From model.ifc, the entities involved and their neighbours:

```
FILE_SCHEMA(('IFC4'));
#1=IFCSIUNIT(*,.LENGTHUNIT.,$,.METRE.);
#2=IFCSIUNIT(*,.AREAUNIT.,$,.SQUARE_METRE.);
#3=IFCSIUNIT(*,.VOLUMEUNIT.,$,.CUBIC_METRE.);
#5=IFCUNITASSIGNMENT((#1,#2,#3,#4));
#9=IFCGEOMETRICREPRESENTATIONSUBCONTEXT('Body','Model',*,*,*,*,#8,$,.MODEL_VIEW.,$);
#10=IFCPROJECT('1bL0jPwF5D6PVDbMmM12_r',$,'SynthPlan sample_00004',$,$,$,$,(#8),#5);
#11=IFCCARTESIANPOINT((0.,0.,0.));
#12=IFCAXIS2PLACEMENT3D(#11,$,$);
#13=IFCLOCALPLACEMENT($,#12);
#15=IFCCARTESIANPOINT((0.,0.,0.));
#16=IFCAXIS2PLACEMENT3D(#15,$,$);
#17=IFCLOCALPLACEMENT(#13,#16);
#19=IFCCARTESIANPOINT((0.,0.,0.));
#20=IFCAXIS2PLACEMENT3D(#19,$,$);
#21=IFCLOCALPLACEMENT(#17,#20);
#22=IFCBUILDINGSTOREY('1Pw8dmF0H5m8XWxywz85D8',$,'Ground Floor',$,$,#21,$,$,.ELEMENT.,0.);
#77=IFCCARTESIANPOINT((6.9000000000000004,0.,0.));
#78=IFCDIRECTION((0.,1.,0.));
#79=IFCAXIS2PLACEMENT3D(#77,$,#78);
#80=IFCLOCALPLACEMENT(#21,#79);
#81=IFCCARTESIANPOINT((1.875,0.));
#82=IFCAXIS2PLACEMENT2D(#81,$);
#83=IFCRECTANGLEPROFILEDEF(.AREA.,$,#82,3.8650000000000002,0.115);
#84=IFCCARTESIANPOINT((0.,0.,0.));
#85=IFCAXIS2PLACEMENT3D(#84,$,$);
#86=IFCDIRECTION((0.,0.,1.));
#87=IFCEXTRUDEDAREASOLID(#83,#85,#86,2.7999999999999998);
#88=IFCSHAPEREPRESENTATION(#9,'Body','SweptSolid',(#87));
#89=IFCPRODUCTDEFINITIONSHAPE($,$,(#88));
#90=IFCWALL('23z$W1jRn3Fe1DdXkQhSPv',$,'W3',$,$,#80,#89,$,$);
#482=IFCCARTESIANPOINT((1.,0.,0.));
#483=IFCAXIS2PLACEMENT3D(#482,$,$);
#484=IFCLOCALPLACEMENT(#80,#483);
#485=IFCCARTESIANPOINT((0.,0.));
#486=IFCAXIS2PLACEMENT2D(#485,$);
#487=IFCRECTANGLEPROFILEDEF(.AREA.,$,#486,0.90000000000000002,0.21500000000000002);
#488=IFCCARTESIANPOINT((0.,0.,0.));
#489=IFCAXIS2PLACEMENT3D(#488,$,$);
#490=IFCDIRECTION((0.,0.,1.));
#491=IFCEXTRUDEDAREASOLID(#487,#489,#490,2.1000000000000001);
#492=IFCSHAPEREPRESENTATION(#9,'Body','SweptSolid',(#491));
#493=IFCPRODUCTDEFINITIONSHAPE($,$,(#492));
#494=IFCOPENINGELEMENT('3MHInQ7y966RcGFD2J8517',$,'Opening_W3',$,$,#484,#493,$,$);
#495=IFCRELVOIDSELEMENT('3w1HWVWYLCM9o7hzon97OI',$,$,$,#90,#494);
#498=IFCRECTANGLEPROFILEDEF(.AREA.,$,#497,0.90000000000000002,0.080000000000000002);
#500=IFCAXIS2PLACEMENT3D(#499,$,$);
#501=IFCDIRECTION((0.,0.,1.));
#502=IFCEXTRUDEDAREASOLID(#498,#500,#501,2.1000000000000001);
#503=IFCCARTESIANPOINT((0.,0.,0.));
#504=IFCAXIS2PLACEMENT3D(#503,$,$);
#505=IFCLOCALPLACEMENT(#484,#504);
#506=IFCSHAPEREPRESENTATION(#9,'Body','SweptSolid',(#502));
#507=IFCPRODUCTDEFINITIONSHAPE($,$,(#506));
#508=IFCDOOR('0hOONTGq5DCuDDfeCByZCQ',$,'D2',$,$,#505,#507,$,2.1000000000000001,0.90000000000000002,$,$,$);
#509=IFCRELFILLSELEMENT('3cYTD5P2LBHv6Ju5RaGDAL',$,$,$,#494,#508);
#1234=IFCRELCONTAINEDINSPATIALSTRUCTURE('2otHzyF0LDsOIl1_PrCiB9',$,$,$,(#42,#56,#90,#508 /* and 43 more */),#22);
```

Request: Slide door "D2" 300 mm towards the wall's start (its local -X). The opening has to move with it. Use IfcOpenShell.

```python
import ifcopenshell
import ifcopenshell.api.geometry
import ifcopenshell.util.placement
import ifcopenshell.util.unit

model = ifcopenshell.open("model.ifc")
unit_scale = ifcopenshell.util.unit.calculate_unit_scale(model)

door = model.by_guid("0hOONTGq5DCuDDfeCByZCQ")
opening = door.FillsVoids[0].RelatingOpeningElement
wall = opening.VoidsElements[0].RelatingBuildingElement

wall_matrix = ifcopenshell.util.placement.get_local_placement(wall.ObjectPlacement)
shift = wall_matrix[:3, 0] * -0.3 / unit_scale
before = ifcopenshell.util.placement.get_local_placement(door.ObjectPlacement)[:3, 3].copy()

# The door is placed relative to its opening, so it follows when the opening moves.
matrix = ifcopenshell.util.placement.get_local_placement(opening.ObjectPlacement)
matrix[:3, 3] += shift
ifcopenshell.api.geometry.edit_object_placement(
    model, product=opening, matrix=matrix, is_si=False, should_transform_children=True
)

after = ifcopenshell.util.placement.get_local_placement(door.ObjectPlacement)[:3, 3]
print("door moved by", (after - before).round(3) + 0.0)

model.write("model_updated.ifc")
```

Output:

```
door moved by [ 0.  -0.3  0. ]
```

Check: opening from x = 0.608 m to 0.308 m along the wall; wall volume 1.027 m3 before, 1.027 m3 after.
